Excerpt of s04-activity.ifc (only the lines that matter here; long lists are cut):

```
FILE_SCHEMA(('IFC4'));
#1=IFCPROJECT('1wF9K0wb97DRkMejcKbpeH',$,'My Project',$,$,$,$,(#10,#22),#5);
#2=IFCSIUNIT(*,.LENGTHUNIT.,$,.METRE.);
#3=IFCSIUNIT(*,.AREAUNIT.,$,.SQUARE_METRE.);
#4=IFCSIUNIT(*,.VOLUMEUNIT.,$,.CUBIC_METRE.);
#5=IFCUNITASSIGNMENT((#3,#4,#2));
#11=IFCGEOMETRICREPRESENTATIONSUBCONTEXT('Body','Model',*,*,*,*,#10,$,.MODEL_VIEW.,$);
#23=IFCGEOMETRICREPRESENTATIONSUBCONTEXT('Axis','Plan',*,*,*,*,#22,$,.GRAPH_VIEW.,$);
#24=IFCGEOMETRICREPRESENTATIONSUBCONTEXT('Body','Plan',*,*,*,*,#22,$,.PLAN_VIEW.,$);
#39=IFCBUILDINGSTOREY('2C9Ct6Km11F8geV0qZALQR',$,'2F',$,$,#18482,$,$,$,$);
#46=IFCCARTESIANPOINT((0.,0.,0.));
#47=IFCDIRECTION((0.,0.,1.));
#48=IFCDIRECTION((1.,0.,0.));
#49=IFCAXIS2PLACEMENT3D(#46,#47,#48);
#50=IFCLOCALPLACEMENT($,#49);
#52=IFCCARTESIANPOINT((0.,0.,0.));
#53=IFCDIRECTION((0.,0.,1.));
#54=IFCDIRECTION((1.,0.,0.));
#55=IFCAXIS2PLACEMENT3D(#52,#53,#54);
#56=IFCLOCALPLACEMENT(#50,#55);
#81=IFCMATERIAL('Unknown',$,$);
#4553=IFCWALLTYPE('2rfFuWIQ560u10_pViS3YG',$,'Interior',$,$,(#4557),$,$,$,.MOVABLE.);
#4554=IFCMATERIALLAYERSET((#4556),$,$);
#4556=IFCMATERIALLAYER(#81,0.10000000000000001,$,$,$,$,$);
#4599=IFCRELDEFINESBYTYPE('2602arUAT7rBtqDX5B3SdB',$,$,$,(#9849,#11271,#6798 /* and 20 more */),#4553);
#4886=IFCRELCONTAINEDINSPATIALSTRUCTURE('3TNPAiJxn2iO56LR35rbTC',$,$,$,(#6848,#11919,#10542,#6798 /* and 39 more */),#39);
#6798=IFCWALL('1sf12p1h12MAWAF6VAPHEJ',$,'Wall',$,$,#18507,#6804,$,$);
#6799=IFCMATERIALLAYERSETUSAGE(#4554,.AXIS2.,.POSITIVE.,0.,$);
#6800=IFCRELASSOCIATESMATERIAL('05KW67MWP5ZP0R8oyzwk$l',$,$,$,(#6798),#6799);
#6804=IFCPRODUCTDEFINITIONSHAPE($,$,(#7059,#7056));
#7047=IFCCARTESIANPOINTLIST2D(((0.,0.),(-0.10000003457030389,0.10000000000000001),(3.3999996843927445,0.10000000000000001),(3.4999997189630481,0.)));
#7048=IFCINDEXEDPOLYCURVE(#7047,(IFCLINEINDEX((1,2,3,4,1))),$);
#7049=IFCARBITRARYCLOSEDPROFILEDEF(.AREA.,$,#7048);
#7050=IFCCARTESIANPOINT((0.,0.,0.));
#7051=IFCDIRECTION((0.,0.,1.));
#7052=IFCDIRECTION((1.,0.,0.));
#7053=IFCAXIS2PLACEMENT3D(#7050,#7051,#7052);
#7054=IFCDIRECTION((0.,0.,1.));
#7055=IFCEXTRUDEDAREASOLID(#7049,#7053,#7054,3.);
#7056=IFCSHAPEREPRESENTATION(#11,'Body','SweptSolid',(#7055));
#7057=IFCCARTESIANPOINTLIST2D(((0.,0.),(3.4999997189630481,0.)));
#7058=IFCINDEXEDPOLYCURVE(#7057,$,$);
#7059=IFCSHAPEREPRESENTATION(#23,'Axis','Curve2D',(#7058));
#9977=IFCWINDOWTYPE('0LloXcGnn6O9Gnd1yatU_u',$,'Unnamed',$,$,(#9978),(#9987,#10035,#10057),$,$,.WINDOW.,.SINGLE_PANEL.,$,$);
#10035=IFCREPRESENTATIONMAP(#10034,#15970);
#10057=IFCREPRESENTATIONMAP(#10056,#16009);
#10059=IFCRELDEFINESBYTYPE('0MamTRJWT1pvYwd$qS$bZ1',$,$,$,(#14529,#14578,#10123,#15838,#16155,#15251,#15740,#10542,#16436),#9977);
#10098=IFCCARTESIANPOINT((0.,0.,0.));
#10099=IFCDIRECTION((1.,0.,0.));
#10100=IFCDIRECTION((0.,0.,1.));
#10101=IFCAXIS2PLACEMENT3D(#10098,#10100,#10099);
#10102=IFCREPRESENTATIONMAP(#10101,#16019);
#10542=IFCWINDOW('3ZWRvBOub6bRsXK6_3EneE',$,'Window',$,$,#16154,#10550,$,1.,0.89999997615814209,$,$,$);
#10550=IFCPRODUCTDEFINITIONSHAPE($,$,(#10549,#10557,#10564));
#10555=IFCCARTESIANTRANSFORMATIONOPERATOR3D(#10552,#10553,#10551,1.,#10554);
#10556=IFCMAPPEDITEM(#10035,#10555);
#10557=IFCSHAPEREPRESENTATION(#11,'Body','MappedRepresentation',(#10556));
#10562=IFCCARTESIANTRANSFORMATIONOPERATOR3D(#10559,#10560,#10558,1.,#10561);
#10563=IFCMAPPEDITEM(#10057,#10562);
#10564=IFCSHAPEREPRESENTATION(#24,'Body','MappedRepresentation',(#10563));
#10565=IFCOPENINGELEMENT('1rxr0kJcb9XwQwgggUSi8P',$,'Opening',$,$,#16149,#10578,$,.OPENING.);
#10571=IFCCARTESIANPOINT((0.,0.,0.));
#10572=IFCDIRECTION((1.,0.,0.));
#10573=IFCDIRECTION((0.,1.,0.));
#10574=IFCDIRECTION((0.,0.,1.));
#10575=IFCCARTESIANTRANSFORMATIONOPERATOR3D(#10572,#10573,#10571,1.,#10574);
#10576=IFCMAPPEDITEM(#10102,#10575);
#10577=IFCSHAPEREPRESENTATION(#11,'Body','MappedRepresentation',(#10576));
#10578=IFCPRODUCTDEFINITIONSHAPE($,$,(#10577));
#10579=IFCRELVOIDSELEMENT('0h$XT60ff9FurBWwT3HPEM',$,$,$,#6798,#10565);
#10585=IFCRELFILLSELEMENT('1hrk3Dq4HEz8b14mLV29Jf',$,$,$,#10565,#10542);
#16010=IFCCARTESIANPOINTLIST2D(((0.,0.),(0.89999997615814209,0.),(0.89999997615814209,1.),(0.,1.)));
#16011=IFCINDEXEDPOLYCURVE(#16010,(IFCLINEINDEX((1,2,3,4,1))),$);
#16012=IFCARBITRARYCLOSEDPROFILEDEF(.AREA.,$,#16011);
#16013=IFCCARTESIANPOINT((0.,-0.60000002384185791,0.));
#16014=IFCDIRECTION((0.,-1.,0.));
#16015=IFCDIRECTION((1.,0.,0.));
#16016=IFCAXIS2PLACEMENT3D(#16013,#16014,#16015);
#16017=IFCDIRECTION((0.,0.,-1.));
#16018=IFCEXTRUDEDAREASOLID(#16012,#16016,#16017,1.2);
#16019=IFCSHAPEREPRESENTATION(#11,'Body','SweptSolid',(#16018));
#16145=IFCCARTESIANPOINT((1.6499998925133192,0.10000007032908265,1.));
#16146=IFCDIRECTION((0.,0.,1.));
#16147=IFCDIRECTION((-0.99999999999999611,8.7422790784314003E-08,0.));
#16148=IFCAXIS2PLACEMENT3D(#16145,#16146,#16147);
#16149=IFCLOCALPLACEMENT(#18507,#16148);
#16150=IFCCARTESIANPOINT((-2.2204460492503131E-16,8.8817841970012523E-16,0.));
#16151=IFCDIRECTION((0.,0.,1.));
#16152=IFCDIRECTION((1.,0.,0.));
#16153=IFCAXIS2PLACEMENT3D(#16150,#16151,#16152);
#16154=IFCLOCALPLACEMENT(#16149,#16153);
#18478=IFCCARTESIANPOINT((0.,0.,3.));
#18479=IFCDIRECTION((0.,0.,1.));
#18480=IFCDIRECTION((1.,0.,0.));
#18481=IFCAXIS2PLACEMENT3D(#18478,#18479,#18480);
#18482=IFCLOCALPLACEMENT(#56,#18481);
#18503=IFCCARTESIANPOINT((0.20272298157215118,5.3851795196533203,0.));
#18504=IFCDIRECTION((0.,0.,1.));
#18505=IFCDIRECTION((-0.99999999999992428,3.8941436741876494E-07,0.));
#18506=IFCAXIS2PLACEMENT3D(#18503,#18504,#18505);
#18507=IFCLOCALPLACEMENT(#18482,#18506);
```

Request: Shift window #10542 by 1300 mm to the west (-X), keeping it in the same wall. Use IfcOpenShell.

```python
import ifcopenshell
import ifcopenshell.api.geometry
import ifcopenshell.util.placement

model = ifcopenshell.open("s04-activity.ifc")

window = model.by_guid("3ZWRvBOub6bRsXK6_3EneE")
opening = window.FillsVoids[0].RelatingOpeningElement
wall = opening.VoidsElements[0].RelatingBuildingElement

wall_matrix = ifcopenshell.util.placement.get_local_placement(wall.ObjectPlacement)
shift = wall_matrix[:3, 0] * 1.3
before = ifcopenshell.util.placement.get_local_placement(window.ObjectPlacement)[:3, 3].copy()

# The window is placed relative to its opening, so it follows when the opening moves.
matrix = ifcopenshell.util.placement.get_local_placement(opening.ObjectPlacement)
matrix[:3, 3] += shift
ifcopenshell.api.geometry.edit_object_placement(
    model, product=opening, matrix=matrix, is_si=False, should_transform_children=True
)

after = ifcopenshell.util.placement.get_local_placement(window.ObjectPlacement)[:3, 3]
print("window moved by", (after - before).round(3) + 0.0)

model.write("s04-activity_v2.ifc")
```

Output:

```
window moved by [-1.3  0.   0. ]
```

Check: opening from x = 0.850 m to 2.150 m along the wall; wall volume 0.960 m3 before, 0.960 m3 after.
